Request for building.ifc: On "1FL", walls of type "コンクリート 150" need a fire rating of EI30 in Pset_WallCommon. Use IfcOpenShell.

First a look at what the model holds.

```python
import ifcopenshell
import ifcopenshell.util.element

model = ifcopenshell.open("building.ifc")
print(model.schema)
storey = next(s for s in model.by_type("IfcBuildingStorey") if s.Name == "1FL")
walls = [e for e in ifcopenshell.util.element.get_decomposition(storey) if e.is_a("IfcWall")]
seen = {}
for e in walls:
    element_type = ifcopenshell.util.element.get_type(e)
    key = (element_type.Name if element_type != e and element_type else None, ifcopenshell.util.element.get_pset(e, "Pset_WallCommon", "FireRating"))
    seen[key] = seen.get(key, 0) + 1
for (name, value), count in sorted(seen.items(), key=str):
    print(count, "x", name, "|", value)
```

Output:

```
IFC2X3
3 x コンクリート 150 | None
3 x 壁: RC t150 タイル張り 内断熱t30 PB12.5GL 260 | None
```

```python
import ifcopenshell
import ifcopenshell.api.pset
import ifcopenshell.util.element

model = ifcopenshell.open("building.ifc")

storey = next(s for s in model.by_type("IfcBuildingStorey") if s.Name == "1FL")
walls = [e for e in ifcopenshell.util.element.get_decomposition(storey) if e.is_a("IfcWall")]

count = 0
for e in walls:
    element_type = ifcopenshell.util.element.get_type(e)
    if element_type in (None, e) or element_type.Name != "コンクリート 150":
        continue
    # add_pset returns the element's existing set when there is one.
    pset = ifcopenshell.api.pset.add_pset(model, product=e, name="Pset_WallCommon")
    ifcopenshell.api.pset.edit_pset(model, pset=pset, properties={"FireRating": "EI30"})
    count += 1

print(count, "walls updated")

model.write("building_rev.ifc")
```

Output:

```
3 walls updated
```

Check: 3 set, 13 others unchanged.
